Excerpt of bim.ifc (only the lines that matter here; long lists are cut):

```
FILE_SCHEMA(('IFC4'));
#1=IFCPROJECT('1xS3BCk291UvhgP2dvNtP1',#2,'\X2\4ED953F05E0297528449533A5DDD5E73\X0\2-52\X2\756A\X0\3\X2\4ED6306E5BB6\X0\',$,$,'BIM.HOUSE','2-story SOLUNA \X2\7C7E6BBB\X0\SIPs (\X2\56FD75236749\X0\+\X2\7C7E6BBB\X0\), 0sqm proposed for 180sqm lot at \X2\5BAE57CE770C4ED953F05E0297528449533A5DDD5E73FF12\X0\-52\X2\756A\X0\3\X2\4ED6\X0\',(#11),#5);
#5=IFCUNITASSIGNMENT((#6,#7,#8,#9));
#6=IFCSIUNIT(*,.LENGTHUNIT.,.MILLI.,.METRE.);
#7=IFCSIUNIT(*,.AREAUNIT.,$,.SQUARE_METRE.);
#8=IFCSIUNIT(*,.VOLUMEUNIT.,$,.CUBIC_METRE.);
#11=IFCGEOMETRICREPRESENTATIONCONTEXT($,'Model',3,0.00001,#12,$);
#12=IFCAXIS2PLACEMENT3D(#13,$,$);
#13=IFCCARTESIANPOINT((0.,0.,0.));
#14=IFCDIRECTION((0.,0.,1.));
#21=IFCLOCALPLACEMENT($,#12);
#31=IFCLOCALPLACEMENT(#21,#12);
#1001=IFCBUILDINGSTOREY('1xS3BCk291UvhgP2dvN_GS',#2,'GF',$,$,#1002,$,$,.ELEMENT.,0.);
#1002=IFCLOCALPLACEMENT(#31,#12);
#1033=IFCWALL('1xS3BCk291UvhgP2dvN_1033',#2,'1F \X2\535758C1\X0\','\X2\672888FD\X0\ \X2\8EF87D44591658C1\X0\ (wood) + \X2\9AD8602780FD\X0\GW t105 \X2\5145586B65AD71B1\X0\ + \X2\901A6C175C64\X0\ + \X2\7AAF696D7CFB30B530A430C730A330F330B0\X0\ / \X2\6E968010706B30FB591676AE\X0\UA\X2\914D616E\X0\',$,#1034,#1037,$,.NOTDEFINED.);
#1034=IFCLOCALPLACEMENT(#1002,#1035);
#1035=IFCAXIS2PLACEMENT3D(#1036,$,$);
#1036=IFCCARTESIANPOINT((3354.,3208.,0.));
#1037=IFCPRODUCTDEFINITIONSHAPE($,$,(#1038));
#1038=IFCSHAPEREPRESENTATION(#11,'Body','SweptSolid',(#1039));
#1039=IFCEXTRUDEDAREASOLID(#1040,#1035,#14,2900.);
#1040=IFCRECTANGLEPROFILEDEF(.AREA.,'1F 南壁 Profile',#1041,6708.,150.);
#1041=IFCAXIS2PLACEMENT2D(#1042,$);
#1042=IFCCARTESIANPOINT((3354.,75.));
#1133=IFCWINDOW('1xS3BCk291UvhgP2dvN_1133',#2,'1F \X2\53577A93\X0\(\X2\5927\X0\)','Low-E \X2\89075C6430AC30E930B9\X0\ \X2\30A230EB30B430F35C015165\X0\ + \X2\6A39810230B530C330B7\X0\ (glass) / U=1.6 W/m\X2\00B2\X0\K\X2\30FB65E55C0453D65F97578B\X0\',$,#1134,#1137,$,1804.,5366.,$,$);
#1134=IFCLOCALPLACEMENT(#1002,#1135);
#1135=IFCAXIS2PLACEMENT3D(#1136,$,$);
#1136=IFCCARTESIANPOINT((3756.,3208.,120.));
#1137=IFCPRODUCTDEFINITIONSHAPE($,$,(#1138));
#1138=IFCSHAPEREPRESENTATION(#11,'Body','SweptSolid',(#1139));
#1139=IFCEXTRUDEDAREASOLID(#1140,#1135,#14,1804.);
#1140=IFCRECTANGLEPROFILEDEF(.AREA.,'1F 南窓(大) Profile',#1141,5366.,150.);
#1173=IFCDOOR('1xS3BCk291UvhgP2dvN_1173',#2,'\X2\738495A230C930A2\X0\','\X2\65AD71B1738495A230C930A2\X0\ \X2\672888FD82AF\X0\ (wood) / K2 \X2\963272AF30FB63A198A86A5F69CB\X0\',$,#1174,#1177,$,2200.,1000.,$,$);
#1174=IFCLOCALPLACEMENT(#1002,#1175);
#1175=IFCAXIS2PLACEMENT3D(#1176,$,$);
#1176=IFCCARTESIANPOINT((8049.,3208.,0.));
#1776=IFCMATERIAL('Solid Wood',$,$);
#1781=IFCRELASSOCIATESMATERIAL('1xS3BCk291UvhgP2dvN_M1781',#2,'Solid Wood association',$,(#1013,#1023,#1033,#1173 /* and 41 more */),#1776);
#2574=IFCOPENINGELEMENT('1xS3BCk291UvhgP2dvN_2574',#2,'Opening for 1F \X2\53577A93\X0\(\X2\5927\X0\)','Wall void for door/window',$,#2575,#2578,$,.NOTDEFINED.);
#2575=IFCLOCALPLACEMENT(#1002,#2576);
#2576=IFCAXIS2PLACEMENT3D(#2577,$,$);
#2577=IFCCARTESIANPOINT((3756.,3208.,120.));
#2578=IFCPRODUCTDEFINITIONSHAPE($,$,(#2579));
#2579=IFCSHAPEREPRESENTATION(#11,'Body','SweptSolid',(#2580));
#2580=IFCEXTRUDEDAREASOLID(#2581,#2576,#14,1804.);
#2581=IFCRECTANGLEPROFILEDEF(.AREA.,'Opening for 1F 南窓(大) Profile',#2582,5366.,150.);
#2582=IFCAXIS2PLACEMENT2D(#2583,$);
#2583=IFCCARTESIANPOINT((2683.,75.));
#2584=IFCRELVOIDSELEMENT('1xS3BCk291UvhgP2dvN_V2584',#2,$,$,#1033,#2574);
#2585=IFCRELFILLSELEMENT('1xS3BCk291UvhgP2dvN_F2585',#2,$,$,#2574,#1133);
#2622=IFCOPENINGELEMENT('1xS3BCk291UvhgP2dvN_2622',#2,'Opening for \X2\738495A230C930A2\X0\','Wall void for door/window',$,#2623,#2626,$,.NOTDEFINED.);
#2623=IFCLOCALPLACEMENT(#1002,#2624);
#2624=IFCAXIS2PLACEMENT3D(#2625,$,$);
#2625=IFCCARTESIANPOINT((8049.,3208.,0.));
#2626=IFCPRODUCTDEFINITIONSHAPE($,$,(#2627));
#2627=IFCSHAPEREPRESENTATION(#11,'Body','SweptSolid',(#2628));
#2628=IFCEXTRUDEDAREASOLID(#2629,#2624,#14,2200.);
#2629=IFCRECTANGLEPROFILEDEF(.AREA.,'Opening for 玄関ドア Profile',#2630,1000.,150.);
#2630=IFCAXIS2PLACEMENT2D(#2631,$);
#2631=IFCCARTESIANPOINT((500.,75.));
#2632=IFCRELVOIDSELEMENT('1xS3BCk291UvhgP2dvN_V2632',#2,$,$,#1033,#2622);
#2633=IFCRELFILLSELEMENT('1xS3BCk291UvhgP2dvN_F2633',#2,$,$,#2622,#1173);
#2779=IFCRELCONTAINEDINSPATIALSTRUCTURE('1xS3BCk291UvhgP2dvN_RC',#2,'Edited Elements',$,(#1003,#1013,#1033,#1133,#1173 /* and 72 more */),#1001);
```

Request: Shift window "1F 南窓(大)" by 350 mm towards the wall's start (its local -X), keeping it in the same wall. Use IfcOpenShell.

```python
import ifcopenshell
import ifcopenshell.api.geometry
import ifcopenshell.util.placement

model = ifcopenshell.open("bim.ifc")

window = model.by_guid("1xS3BCk291UvhgP2dvN_1133")
opening = window.FillsVoids[0].RelatingOpeningElement
wall = opening.VoidsElements[0].RelatingBuildingElement

wall_matrix = ifcopenshell.util.placement.get_local_placement(wall.ObjectPlacement)
shift = wall_matrix[:3, 0] * -350.0
before = ifcopenshell.util.placement.get_local_placement(window.ObjectPlacement)[:3, 3].copy()

# The window is not placed relative to its opening, so move both.
for product in (opening, window):
    matrix = ifcopenshell.util.placement.get_local_placement(product.ObjectPlacement)
    matrix[:3, 3] += shift
    ifcopenshell.api.geometry.edit_object_placement(model, product=product, matrix=matrix, is_si=False)

after = ifcopenshell.util.placement.get_local_placement(window.ObjectPlacement)[:3, 3]
print("window moved by", (after - before).round(3) + 0.0)

model.write("bim_v2.ifc")
```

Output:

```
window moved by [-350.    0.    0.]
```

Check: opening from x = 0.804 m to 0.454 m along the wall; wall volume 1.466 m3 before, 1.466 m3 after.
